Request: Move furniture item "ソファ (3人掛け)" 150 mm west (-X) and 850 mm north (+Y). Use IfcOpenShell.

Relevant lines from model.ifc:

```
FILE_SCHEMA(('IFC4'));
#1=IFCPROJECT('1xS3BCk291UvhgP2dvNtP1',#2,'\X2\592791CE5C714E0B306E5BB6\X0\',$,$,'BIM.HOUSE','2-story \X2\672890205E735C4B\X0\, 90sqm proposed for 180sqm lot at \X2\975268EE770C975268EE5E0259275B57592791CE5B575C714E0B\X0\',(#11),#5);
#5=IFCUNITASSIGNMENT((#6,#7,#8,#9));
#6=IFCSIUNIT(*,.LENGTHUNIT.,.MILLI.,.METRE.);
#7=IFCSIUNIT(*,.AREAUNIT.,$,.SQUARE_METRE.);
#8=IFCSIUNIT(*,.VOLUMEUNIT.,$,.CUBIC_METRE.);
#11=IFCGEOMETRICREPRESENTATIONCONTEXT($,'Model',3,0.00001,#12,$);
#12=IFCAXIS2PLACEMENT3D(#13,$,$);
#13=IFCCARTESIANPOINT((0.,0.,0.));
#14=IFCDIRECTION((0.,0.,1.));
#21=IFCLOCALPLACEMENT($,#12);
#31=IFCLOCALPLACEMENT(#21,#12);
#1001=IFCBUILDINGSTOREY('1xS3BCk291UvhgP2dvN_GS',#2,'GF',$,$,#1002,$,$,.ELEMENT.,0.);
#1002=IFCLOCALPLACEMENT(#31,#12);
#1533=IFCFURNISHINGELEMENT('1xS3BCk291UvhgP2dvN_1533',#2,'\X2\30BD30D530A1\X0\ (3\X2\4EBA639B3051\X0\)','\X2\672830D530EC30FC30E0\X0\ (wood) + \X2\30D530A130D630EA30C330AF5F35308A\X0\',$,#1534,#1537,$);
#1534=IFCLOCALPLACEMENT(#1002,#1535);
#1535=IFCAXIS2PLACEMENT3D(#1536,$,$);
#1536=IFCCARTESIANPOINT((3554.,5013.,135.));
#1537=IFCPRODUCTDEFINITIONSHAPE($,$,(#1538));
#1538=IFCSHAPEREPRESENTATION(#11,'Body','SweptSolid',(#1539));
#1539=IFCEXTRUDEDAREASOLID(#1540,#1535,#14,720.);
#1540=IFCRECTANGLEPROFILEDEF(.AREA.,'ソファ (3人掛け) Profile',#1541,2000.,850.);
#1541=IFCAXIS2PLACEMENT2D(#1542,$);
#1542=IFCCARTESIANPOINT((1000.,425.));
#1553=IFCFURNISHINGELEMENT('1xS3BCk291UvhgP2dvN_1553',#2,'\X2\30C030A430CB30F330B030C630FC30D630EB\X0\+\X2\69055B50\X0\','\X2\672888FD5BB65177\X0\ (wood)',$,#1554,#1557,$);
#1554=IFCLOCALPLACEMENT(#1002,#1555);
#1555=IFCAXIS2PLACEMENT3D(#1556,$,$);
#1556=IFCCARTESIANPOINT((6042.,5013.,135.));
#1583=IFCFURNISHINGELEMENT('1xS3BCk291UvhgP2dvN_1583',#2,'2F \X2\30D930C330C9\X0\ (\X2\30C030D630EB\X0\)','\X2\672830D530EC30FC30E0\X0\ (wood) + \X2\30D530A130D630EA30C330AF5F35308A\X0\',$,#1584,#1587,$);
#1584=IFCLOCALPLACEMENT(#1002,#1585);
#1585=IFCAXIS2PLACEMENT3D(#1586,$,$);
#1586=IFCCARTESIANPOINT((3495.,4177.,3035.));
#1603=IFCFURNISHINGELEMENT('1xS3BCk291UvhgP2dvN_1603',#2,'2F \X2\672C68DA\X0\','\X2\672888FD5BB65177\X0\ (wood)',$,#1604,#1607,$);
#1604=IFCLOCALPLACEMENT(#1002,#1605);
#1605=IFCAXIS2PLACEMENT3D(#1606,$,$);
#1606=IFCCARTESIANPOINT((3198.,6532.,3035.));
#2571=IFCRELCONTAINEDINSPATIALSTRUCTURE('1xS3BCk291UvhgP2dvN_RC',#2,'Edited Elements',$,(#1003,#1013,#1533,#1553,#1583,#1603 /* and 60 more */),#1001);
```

```python
import ifcopenshell
import ifcopenshell.api.geometry
import ifcopenshell.util.placement
import ifcopenshell.util.unit

model = ifcopenshell.open("model.ifc")
unit_scale = ifcopenshell.util.unit.calculate_unit_scale(model)

item = model.by_guid("1xS3BCk291UvhgP2dvN_1533")
matrix = ifcopenshell.util.placement.get_local_placement(item.ObjectPlacement)
matrix[0, 3] -= 0.15 / unit_scale
matrix[1, 3] += 0.85 / unit_scale
ifcopenshell.api.geometry.edit_object_placement(model, product=item, matrix=matrix, is_si=False)

print(ifcopenshell.util.placement.get_local_placement(item.ObjectPlacement).round(3) + 0.0)

model.write("model-out.ifc")
```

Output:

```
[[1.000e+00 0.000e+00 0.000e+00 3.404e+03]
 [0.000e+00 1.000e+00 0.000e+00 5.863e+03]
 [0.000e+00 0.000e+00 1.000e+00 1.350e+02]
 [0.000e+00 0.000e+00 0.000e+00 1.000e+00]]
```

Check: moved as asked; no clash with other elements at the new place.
